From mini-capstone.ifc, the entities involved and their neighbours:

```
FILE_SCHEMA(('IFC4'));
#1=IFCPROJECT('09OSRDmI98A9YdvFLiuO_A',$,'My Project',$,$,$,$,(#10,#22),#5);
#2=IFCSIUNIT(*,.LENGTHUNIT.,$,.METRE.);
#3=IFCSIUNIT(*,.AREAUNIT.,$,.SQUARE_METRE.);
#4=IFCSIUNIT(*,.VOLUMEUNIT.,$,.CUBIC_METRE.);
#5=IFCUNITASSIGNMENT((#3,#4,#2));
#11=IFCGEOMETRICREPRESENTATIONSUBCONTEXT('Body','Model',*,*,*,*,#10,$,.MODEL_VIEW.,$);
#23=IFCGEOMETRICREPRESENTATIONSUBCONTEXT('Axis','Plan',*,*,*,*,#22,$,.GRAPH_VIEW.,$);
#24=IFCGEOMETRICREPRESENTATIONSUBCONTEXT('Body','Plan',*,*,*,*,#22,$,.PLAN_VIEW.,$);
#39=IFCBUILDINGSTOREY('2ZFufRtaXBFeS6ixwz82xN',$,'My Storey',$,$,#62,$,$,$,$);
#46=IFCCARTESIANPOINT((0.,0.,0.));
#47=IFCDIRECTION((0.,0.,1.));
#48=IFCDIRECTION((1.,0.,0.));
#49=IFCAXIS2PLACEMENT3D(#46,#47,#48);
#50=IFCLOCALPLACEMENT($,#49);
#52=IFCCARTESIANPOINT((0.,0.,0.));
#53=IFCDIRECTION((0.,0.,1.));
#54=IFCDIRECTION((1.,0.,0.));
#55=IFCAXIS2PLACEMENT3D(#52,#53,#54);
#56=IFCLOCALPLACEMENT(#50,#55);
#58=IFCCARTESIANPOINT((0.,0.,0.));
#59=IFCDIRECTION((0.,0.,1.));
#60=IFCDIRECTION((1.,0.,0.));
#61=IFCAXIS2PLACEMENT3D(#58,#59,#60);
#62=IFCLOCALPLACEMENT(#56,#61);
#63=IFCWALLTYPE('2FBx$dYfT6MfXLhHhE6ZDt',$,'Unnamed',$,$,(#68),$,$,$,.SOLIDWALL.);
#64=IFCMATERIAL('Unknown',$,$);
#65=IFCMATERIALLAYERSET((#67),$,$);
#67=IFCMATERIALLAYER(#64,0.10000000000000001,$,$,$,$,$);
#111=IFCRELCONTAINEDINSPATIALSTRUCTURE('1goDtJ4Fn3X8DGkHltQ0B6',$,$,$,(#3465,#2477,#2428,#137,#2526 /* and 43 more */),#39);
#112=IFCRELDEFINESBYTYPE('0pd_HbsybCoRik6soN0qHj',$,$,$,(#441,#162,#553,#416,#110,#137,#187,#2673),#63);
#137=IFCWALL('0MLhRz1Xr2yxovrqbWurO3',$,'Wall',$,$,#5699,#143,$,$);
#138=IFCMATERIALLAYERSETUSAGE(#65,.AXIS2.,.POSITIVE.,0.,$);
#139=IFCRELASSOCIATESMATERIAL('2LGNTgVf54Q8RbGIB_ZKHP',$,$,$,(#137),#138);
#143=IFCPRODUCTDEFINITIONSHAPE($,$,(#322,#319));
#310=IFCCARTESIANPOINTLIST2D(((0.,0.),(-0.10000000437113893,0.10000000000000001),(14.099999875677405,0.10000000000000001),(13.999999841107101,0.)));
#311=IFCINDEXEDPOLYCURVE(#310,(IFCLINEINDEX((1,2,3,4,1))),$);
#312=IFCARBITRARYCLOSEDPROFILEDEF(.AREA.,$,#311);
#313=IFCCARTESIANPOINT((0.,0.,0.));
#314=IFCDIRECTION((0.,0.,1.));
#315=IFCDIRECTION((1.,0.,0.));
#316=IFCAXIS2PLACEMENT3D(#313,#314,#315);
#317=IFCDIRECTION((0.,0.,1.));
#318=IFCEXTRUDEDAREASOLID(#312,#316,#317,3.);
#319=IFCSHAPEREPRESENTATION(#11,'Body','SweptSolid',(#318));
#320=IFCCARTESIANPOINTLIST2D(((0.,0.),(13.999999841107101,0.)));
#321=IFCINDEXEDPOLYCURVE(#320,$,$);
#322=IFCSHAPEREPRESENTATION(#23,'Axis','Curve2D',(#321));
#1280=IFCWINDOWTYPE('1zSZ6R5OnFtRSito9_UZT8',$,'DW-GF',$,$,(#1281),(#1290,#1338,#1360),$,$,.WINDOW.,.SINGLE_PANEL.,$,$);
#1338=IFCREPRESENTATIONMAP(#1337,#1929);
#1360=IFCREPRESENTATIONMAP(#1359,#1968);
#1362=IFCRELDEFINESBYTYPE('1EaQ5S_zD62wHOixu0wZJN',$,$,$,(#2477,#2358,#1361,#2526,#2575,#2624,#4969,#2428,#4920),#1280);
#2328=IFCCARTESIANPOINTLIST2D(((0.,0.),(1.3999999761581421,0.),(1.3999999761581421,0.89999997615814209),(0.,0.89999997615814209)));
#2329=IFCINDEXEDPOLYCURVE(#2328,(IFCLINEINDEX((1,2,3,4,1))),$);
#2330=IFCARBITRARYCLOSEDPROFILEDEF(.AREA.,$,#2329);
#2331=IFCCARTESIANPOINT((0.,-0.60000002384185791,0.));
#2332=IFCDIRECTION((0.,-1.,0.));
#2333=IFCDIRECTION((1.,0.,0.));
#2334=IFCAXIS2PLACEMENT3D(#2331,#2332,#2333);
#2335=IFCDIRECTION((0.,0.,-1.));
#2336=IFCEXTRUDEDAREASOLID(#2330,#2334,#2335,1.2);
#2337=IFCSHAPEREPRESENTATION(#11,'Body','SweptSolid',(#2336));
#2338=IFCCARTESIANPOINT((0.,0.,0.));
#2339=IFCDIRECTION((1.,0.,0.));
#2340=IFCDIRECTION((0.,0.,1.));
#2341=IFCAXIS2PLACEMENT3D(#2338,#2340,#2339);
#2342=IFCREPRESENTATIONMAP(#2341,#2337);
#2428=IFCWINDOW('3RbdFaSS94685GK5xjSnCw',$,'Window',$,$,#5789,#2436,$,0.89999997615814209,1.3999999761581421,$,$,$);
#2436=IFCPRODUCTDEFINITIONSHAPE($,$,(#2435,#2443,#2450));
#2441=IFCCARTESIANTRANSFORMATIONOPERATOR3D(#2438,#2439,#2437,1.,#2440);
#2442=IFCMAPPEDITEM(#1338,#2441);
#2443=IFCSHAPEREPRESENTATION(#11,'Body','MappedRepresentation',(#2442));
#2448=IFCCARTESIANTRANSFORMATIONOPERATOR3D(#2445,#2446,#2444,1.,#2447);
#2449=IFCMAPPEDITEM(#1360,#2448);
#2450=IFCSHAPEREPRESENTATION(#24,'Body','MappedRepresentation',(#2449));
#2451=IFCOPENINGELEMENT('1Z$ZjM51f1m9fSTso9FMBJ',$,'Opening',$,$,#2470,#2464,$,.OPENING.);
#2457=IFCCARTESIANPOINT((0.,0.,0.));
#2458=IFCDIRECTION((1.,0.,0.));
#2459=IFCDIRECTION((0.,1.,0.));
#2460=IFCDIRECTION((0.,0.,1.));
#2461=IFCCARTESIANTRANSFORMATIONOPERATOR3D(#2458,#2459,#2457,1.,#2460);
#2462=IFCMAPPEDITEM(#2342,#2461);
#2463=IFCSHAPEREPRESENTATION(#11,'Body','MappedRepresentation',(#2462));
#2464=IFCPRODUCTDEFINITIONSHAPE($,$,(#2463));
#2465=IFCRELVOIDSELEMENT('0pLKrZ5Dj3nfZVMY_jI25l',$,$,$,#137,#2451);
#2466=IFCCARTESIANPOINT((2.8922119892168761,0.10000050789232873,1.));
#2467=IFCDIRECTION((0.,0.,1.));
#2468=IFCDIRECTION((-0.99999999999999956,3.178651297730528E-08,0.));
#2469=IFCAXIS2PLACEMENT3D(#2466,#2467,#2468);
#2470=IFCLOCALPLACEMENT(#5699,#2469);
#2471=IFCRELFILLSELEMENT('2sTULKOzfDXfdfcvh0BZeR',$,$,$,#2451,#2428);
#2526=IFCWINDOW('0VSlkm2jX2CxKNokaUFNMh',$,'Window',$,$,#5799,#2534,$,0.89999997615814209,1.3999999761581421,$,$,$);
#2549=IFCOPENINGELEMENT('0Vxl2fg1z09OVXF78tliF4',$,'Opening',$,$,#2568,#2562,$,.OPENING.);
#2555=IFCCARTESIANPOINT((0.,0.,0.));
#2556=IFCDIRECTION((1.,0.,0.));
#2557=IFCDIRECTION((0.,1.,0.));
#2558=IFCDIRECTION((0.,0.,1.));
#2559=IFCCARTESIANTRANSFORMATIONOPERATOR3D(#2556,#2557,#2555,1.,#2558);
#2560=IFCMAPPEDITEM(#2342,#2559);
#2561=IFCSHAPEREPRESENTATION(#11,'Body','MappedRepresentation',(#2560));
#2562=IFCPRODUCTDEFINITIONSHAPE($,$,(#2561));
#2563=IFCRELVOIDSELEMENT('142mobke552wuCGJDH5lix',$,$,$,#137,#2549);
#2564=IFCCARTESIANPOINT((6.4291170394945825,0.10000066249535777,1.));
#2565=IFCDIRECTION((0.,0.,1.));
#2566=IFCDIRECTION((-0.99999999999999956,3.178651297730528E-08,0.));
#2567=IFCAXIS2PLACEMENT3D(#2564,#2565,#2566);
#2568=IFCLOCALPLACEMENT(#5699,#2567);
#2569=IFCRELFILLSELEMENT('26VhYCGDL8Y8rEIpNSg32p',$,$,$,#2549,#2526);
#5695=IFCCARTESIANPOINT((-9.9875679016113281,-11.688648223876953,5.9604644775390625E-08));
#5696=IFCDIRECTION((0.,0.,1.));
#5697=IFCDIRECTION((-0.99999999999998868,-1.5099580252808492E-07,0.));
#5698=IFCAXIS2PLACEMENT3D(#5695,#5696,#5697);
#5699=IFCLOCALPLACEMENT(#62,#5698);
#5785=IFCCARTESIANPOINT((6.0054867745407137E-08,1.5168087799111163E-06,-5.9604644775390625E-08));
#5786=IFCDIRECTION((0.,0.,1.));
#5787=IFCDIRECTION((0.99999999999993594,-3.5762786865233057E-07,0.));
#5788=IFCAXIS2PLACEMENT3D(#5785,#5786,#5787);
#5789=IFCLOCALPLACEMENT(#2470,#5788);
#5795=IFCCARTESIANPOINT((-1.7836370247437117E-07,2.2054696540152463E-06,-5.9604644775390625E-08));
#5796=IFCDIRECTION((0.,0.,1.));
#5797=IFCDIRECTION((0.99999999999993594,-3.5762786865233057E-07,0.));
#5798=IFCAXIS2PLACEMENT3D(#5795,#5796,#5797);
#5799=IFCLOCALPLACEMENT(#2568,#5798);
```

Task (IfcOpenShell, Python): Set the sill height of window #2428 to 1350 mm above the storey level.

```python
import numpy as np
import ifcopenshell
import ifcopenshell.api.geometry
import ifcopenshell.geom
import ifcopenshell.util.element
import ifcopenshell.util.placement
import ifcopenshell.util.shape
import ifcopenshell.util.unit

model = ifcopenshell.open("mini-capstone.ifc")
unit_scale = ifcopenshell.util.unit.calculate_unit_scale(model)

window = model.by_guid("3RbdFaSS94685GK5xjSnCw")
opening = window.FillsVoids[0].RelatingOpeningElement
storey = ifcopenshell.util.element.get_container(window, ifc_class="IfcBuildingStorey")
level = ifcopenshell.util.placement.get_local_placement(storey.ObjectPlacement)[2, 3]

# The opening's origin need not be at the sill, so measure its lowest point.
shape = ifcopenshell.geom.create_shape(ifcopenshell.geom.settings(), opening)
bottom = ifcopenshell.util.shape.get_shape_bottom_elevation(shape, shape.geometry) / unit_scale
dz = level + 1.35 / unit_scale - bottom

shift = np.array([0.0, 0.0, dz])
# The window is placed relative to its opening, so it follows when the opening moves.
matrix = ifcopenshell.util.placement.get_local_placement(opening.ObjectPlacement)
matrix[:3, 3] += shift
ifcopenshell.api.geometry.edit_object_placement(
    model, product=opening, matrix=matrix, is_si=False, should_transform_children=True
)

print(f"moved by {dz * unit_scale:+.3f} m")

model.write("mini-capstone_updated.ifc")
```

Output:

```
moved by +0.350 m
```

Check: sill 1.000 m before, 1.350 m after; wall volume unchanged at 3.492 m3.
